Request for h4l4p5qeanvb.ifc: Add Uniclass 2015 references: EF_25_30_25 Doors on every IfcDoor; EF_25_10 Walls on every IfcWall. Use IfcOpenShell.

First a look at what the model holds.

```python
import ifcopenshell

model = ifcopenshell.open("h4l4p5qeanvb.ifc")
print(model.schema)
print("classifications:", [c.Name for c in model.by_type("IfcClassification")])
for ifc_class in ("IfcDoor", "IfcRoof", "IfcStair", "IfcWall", "IfcWindow"):
    print(ifc_class, len(model.by_type(ifc_class)))
```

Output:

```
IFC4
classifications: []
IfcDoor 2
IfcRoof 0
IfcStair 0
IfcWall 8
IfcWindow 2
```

```python
import ifcopenshell
import ifcopenshell.api.classification

model = ifcopenshell.open("h4l4p5qeanvb.ifc")

system = ifcopenshell.api.classification.add_classification(model, classification="Uniclass 2015")

codes = {
    "IfcDoor": ("EF_25_30_25", "Doors"),
    "IfcWall": ("EF_25_10", "Walls"),
}
for ifc_class, (code, name) in codes.items():
    products = model.by_type(ifc_class)
    ifcopenshell.api.classification.add_reference(
        model, products=products, classification=system, identification=code, name=name
    )
    print(code, len(products))

model.write("h4l4p5qeanvb_updated.ifc")
```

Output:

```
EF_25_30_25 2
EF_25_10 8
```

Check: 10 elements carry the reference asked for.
